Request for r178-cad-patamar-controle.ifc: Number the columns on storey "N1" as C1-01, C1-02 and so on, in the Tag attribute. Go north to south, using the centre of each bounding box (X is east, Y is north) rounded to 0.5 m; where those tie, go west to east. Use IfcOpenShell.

First a look at what the model holds.

```python
import ifcopenshell
import ifcopenshell.util.element
import ifcopenshell.util.placement

model = ifcopenshell.open("r178-cad-patamar-controle.ifc")
print(model.schema)
storey = next(s for s in model.by_type("IfcBuildingStorey") if s.Name == "N1")
columns = [e for e in ifcopenshell.util.element.get_decomposition(storey) if e.is_a("IfcColumn")]
for e in sorted(columns, key=lambda e: e.id()):
    origin = ifcopenshell.util.placement.get_local_placement(e.ObjectPlacement)[:3, 3]
    print(e.id(), e.Tag, e.Name, origin.round(2) + 0.0, sep=" | ")
```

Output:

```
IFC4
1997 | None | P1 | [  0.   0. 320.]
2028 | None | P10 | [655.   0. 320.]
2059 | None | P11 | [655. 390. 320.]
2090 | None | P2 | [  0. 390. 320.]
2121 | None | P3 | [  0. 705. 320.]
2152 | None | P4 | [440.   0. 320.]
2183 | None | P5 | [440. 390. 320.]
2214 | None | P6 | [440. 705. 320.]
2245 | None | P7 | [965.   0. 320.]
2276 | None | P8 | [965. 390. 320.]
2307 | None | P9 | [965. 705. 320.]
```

```python
import ifcopenshell
import ifcopenshell.geom
import ifcopenshell.util.element
import ifcopenshell.util.shape

model = ifcopenshell.open("r178-cad-patamar-controle.ifc")
settings = ifcopenshell.geom.settings()
settings.set("use-world-coords", True)


def centre(element):
    shape = ifcopenshell.geom.create_shape(settings, element)
    return ifcopenshell.util.shape.get_bbox_centroid(shape.geometry)


storey = next(s for s in model.by_type("IfcBuildingStorey") if s.Name == "N1")
columns = [e for e in ifcopenshell.util.element.get_decomposition(storey) if e.is_a("IfcColumn")]

# Insertion points can sit at a corner or the storey origin, so sort by the geometry (in metres).
centres = {e: centre(e) for e in columns}
columns.sort(key=lambda e: (-round(centres[e][1] / 0.5), centres[e][0]))

for i, e in enumerate(columns, start=1):
    number = f"C1-{i:02d}"
    e.Tag = number
    print(e.id(), number)

model.write("r178-cad-patamar-controle_edited.ifc")
```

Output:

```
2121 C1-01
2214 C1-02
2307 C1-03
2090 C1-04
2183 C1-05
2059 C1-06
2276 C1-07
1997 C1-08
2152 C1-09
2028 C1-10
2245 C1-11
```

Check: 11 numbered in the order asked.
